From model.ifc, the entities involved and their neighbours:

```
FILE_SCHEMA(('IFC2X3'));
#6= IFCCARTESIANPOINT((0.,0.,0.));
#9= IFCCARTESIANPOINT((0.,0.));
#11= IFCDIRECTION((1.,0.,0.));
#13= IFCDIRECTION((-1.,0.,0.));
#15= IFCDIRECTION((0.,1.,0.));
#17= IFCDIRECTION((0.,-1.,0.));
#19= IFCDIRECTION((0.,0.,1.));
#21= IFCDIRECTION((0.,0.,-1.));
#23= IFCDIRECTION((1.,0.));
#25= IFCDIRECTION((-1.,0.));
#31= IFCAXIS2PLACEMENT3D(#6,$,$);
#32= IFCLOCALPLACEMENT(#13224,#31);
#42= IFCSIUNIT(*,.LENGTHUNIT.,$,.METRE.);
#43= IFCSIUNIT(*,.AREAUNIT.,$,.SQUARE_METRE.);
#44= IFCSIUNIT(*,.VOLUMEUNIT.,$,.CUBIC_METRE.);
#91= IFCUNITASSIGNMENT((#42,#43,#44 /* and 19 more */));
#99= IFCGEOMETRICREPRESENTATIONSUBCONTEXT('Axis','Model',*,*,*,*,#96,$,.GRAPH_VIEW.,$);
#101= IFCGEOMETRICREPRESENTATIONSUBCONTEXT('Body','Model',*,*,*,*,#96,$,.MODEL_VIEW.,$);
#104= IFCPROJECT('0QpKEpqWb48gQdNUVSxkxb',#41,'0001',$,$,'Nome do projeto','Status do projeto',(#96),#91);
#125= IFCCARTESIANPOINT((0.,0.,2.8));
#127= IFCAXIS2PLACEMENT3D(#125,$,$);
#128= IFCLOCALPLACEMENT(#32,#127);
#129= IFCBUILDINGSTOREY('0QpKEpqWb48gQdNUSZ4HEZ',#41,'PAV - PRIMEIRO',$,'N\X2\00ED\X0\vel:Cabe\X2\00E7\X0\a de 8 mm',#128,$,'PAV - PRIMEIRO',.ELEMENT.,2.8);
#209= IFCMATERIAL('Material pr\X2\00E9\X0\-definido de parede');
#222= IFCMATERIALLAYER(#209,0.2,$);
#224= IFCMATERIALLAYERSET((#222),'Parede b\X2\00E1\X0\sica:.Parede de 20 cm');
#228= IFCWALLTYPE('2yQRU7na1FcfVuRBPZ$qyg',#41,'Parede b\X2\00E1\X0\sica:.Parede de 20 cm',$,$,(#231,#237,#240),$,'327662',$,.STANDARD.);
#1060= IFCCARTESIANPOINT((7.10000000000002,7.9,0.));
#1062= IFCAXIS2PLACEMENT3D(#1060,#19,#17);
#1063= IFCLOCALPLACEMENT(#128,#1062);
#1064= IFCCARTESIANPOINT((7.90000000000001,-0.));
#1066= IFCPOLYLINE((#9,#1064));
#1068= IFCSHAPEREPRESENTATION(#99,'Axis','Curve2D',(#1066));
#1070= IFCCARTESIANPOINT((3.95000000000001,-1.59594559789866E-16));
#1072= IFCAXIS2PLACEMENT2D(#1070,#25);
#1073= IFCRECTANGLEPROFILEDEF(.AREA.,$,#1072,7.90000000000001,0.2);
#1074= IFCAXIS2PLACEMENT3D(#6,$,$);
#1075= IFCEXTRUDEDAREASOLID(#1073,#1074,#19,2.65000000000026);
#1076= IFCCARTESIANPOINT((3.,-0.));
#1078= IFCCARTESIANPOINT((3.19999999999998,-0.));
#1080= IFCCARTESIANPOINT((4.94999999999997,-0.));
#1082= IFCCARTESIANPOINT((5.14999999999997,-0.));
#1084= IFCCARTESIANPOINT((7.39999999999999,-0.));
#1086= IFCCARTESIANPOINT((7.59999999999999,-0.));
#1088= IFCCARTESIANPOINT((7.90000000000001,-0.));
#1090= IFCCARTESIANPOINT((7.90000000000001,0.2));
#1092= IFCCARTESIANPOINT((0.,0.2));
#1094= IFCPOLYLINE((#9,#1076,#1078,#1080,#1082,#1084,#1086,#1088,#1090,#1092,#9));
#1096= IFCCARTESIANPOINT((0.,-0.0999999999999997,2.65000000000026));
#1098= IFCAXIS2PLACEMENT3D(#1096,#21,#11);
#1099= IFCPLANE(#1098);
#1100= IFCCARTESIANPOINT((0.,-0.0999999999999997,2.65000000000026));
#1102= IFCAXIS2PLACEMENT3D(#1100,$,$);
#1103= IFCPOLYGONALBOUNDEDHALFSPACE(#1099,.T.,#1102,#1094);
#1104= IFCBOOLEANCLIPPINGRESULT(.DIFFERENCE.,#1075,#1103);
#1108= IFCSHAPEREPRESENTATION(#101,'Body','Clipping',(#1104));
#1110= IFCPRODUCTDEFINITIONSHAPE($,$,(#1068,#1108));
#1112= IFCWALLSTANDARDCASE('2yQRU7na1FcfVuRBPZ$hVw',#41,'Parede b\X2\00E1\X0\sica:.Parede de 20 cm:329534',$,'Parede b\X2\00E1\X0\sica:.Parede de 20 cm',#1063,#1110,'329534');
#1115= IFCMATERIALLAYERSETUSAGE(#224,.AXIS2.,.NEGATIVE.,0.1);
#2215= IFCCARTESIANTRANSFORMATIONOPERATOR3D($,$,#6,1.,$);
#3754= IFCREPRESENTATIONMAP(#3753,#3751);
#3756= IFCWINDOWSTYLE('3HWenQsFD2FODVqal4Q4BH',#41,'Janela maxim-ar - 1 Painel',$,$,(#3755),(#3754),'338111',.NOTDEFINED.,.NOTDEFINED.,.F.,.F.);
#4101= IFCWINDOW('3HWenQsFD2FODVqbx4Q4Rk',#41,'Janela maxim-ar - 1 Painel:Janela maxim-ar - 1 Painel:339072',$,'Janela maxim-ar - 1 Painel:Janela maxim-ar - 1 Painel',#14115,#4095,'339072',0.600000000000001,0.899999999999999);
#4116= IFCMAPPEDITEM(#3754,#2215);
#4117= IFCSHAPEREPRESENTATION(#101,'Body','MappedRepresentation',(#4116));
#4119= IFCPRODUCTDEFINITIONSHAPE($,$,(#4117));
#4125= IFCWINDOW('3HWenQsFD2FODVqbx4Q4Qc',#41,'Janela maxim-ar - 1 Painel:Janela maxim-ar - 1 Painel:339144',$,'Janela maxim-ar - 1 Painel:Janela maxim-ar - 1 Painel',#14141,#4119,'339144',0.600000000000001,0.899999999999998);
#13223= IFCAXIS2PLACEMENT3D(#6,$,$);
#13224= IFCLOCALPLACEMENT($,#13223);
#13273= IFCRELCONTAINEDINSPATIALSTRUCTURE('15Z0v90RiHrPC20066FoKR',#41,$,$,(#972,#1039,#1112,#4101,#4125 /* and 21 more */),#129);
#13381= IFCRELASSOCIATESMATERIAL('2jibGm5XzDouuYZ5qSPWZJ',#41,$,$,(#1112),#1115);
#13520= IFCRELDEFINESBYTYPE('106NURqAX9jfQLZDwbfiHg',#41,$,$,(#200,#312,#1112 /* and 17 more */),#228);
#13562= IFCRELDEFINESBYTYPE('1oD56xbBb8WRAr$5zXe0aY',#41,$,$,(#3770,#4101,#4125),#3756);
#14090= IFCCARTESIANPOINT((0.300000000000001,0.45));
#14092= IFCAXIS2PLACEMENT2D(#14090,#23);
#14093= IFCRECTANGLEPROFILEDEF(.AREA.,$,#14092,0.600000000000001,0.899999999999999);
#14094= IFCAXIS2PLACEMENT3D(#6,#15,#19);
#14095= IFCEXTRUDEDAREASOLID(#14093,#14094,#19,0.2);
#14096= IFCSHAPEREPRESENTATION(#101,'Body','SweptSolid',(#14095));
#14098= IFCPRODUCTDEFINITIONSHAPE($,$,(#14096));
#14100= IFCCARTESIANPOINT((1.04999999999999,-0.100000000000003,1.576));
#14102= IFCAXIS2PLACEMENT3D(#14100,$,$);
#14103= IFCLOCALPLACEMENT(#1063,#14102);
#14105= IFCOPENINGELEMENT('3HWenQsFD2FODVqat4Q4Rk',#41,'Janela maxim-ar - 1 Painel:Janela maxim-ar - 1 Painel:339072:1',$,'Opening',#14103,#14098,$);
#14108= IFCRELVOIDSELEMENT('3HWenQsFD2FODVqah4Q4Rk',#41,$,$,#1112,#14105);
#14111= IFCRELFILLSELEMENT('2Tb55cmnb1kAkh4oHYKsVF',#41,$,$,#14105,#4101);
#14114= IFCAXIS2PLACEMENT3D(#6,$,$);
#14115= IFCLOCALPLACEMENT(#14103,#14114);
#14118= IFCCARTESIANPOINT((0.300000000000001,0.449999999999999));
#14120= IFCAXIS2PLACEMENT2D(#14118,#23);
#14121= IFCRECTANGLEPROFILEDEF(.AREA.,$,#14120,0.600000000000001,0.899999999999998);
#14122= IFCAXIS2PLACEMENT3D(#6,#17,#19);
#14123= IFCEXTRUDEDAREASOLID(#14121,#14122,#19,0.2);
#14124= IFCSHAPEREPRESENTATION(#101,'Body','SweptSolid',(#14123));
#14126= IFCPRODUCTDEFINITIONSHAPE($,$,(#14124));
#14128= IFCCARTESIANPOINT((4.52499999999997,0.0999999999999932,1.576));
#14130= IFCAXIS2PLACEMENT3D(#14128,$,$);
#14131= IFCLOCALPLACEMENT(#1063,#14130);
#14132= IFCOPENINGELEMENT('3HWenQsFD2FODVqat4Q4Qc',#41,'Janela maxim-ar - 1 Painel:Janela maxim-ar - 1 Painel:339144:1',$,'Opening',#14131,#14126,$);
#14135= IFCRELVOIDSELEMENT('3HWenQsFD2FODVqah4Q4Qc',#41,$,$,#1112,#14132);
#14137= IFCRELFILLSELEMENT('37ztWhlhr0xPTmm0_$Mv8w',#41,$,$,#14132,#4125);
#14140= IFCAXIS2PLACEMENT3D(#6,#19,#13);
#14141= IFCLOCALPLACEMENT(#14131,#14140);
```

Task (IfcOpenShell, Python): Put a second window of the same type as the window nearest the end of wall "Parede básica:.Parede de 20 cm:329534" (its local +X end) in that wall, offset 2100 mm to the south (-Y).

```python
import ifcopenshell
import ifcopenshell.api.feature
import ifcopenshell.api.geometry
import ifcopenshell.api.root
import ifcopenshell.geom
import ifcopenshell.util.element
import ifcopenshell.util.placement
import ifcopenshell.util.shape

model = ifcopenshell.open("model.ifc")
settings = ifcopenshell.geom.settings()


def volume(element):
    """Net volume in cubic metres, openings subtracted."""
    shape = ifcopenshell.geom.create_shape(settings, element)
    return ifcopenshell.util.shape.get_volume(shape.geometry)


def reuse_history(source, copy):
    """copy_class also copies each property set's owner history, people and application; keep the originals."""
    for rel in copy.IsDefinedBy:
        if rel.is_a("IfcRelDefinesByProperties") and (history := rel.RelatingPropertyDefinition.OwnerHistory):
            rel.RelatingPropertyDefinition.OwnerHistory = source.OwnerHistory
            ifcopenshell.util.element.remove_deep2(model, history)


window = model.by_guid("3HWenQsFD2FODVqbx4Q4Qc")
opening = window.FillsVoids[0].RelatingOpeningElement
wall = opening.VoidsElements[0].RelatingBuildingElement
before = volume(wall)
shift = ifcopenshell.util.placement.get_local_placement(wall.ObjectPlacement)[:3, 0] * 2.1

# copy_class copies the void relationship, type, container and properties, but no geometry.
new_opening = ifcopenshell.api.root.copy_class(model, product=opening)
new_opening.Representation = ifcopenshell.util.element.copy_deep(
    model, opening.Representation, exclude=["IfcGeometricRepresentationContext", "IfcRepresentationMap"]
)
new_opening.Name = "Janela maxim-ar - 1 Painel:Janela maxim-ar - 1 Painel"
new_window = ifcopenshell.api.root.copy_class(model, product=window)
new_window.Representation = ifcopenshell.util.element.copy_deep(
    model, window.Representation, exclude=["IfcGeometricRepresentationContext", "IfcRepresentationMap"]
)
new_window.Name = "Janela maxim-ar - 1 Painel:Janela maxim-ar - 1 Painel"
new_window.Tag = None
reuse_history(window, new_window)
fills = ifcopenshell.api.feature.add_filling(model, opening=new_opening, element=new_window)
fills.OwnerHistory = new_window.OwnerHistory  # required in IFC2X3

for old, new in ((opening, new_opening), (window, new_window)):
    matrix = ifcopenshell.util.placement.get_local_placement(old.ObjectPlacement)
    matrix[:3, 3] += shift
    ifcopenshell.api.geometry.edit_object_placement(model, product=new, matrix=matrix, is_si=False)

after = volume(wall)

print(f"wall volume {before:.3f} -> {after:.3f} m3")

model.write("model_rev.ifc")
```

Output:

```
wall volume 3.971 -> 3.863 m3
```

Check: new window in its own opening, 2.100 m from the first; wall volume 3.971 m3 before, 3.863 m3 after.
